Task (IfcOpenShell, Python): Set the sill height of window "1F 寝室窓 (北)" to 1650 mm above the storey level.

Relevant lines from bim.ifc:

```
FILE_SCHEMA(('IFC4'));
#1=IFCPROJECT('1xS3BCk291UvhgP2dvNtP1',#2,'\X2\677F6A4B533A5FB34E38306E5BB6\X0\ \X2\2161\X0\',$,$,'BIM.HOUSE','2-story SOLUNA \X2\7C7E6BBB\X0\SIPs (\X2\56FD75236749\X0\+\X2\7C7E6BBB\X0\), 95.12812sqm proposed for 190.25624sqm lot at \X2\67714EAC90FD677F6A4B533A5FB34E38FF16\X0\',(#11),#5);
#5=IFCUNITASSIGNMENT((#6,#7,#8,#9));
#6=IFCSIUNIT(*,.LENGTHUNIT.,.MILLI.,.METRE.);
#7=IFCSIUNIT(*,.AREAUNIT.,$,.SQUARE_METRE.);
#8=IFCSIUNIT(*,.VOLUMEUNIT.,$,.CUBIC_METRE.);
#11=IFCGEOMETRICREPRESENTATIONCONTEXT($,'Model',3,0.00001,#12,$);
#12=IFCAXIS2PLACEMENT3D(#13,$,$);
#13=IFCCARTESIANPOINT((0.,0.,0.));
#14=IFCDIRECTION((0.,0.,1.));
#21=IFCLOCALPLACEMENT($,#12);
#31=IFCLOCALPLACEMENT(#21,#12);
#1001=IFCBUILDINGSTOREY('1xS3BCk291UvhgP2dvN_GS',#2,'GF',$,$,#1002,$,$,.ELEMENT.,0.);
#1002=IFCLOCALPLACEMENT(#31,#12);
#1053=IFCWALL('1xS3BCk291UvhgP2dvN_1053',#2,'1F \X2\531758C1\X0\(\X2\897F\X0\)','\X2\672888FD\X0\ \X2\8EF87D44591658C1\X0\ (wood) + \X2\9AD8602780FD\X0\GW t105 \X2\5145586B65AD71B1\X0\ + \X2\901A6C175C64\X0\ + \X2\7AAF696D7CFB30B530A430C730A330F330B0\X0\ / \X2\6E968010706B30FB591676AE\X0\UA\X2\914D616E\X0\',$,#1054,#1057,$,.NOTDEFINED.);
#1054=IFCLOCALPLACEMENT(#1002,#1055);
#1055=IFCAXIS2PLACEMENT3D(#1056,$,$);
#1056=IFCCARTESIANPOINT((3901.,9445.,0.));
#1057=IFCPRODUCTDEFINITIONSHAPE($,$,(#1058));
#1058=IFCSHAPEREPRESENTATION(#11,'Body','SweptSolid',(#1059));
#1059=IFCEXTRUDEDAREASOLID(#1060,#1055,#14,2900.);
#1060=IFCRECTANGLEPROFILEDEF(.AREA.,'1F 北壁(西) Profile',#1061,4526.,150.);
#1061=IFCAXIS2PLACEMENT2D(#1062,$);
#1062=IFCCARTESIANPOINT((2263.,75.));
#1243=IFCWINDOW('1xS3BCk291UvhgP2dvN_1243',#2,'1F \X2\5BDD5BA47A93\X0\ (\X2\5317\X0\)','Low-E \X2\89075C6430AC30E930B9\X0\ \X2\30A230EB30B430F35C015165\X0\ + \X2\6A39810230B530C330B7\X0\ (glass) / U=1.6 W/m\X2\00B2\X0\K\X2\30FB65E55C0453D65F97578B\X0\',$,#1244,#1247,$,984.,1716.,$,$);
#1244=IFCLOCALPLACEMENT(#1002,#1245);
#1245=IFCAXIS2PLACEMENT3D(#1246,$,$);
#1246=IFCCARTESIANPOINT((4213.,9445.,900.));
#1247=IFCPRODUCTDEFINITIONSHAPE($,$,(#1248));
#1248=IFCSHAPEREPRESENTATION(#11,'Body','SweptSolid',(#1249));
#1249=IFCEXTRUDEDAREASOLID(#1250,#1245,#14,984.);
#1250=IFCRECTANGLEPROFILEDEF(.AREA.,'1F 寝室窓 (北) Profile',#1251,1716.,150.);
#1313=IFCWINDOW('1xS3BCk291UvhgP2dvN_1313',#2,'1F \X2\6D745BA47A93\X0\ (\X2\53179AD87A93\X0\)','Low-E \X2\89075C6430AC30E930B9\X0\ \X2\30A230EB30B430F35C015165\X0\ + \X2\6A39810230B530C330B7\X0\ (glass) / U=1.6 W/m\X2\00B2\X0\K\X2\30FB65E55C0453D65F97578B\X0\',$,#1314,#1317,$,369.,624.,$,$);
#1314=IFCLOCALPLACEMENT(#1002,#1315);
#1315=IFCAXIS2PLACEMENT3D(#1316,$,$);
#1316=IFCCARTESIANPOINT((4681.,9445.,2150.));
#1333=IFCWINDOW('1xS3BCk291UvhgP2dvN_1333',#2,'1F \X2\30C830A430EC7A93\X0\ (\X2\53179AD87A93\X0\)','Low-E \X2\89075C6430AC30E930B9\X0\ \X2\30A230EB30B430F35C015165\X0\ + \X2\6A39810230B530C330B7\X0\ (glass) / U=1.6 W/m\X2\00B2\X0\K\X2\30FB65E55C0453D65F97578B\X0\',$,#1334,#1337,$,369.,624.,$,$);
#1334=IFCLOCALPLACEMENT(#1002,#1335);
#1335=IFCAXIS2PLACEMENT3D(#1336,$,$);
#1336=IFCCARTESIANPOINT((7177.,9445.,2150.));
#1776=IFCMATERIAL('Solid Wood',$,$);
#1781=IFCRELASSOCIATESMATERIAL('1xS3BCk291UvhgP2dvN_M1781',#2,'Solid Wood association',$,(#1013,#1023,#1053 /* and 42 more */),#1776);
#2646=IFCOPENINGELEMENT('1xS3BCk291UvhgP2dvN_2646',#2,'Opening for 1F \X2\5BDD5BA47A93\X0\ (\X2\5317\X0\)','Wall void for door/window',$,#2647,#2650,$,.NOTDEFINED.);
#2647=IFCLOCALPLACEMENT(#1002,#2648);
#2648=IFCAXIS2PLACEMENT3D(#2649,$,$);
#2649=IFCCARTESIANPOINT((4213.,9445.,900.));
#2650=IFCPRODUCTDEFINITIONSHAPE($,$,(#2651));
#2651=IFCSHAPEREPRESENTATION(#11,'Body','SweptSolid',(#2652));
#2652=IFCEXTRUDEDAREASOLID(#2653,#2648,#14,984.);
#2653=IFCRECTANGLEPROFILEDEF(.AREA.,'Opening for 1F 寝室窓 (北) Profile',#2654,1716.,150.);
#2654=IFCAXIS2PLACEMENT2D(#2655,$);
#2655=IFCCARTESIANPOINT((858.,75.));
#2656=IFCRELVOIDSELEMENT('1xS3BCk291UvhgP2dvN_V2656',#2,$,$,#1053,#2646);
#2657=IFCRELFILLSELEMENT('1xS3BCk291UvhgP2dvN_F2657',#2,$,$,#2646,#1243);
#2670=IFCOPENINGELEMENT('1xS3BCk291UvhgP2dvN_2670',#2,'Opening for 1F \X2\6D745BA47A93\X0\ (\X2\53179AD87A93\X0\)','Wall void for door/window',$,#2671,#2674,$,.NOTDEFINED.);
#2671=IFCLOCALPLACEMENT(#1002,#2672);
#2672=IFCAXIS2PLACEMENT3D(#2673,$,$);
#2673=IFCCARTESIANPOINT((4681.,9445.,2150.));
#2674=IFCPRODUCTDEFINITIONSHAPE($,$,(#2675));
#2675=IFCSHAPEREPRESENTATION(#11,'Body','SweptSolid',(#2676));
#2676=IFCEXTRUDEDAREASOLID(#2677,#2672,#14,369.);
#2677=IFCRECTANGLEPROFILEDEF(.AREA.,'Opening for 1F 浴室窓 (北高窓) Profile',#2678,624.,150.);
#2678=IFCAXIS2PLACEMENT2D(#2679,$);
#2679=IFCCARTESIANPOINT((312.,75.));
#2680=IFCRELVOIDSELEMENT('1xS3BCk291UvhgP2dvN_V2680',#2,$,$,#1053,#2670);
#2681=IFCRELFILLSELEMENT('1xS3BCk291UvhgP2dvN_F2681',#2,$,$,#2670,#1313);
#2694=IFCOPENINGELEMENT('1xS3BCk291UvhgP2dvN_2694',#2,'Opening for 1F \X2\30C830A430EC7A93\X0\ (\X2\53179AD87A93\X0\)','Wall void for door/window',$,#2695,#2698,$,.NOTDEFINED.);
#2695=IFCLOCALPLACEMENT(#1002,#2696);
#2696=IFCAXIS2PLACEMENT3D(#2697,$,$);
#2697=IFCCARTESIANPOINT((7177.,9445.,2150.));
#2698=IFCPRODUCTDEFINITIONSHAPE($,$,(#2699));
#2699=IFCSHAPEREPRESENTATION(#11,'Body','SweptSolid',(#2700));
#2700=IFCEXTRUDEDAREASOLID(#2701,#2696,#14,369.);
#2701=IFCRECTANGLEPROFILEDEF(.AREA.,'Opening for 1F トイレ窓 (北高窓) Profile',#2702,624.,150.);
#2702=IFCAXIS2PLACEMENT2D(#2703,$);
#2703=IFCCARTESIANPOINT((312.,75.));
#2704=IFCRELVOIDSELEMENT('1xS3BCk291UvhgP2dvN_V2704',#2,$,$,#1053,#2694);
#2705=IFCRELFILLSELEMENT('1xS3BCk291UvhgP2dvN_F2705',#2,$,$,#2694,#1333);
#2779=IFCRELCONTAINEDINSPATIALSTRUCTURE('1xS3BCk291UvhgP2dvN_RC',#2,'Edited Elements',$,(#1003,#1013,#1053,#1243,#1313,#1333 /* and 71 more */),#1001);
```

```python
import numpy as np
import ifcopenshell
import ifcopenshell.api.geometry
import ifcopenshell.geom
import ifcopenshell.util.element
import ifcopenshell.util.placement
import ifcopenshell.util.shape
import ifcopenshell.util.unit

model = ifcopenshell.open("bim.ifc")
unit_scale = ifcopenshell.util.unit.calculate_unit_scale(model)

window = model.by_guid("1xS3BCk291UvhgP2dvN_1243")
opening = window.FillsVoids[0].RelatingOpeningElement
storey = ifcopenshell.util.element.get_container(window, ifc_class="IfcBuildingStorey")
level = ifcopenshell.util.placement.get_local_placement(storey.ObjectPlacement)[2, 3]

# The opening's origin need not be at the sill, so measure its lowest point.
shape = ifcopenshell.geom.create_shape(ifcopenshell.geom.settings(), opening)
bottom = ifcopenshell.util.shape.get_shape_bottom_elevation(shape, shape.geometry) / unit_scale
dz = level + 1.65 / unit_scale - bottom

shift = np.array([0.0, 0.0, dz])
# The window is not placed relative to its opening, so move both.
for product in (opening, window):
    matrix = ifcopenshell.util.placement.get_local_placement(product.ObjectPlacement)
    matrix[:3, 3] += shift
    ifcopenshell.api.geometry.edit_object_placement(model, product=product, matrix=matrix, is_si=False)

print(f"moved by {dz * unit_scale:+.3f} m")

model.write("bim_edited.ifc")
```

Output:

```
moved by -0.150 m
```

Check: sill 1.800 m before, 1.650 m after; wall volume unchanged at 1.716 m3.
